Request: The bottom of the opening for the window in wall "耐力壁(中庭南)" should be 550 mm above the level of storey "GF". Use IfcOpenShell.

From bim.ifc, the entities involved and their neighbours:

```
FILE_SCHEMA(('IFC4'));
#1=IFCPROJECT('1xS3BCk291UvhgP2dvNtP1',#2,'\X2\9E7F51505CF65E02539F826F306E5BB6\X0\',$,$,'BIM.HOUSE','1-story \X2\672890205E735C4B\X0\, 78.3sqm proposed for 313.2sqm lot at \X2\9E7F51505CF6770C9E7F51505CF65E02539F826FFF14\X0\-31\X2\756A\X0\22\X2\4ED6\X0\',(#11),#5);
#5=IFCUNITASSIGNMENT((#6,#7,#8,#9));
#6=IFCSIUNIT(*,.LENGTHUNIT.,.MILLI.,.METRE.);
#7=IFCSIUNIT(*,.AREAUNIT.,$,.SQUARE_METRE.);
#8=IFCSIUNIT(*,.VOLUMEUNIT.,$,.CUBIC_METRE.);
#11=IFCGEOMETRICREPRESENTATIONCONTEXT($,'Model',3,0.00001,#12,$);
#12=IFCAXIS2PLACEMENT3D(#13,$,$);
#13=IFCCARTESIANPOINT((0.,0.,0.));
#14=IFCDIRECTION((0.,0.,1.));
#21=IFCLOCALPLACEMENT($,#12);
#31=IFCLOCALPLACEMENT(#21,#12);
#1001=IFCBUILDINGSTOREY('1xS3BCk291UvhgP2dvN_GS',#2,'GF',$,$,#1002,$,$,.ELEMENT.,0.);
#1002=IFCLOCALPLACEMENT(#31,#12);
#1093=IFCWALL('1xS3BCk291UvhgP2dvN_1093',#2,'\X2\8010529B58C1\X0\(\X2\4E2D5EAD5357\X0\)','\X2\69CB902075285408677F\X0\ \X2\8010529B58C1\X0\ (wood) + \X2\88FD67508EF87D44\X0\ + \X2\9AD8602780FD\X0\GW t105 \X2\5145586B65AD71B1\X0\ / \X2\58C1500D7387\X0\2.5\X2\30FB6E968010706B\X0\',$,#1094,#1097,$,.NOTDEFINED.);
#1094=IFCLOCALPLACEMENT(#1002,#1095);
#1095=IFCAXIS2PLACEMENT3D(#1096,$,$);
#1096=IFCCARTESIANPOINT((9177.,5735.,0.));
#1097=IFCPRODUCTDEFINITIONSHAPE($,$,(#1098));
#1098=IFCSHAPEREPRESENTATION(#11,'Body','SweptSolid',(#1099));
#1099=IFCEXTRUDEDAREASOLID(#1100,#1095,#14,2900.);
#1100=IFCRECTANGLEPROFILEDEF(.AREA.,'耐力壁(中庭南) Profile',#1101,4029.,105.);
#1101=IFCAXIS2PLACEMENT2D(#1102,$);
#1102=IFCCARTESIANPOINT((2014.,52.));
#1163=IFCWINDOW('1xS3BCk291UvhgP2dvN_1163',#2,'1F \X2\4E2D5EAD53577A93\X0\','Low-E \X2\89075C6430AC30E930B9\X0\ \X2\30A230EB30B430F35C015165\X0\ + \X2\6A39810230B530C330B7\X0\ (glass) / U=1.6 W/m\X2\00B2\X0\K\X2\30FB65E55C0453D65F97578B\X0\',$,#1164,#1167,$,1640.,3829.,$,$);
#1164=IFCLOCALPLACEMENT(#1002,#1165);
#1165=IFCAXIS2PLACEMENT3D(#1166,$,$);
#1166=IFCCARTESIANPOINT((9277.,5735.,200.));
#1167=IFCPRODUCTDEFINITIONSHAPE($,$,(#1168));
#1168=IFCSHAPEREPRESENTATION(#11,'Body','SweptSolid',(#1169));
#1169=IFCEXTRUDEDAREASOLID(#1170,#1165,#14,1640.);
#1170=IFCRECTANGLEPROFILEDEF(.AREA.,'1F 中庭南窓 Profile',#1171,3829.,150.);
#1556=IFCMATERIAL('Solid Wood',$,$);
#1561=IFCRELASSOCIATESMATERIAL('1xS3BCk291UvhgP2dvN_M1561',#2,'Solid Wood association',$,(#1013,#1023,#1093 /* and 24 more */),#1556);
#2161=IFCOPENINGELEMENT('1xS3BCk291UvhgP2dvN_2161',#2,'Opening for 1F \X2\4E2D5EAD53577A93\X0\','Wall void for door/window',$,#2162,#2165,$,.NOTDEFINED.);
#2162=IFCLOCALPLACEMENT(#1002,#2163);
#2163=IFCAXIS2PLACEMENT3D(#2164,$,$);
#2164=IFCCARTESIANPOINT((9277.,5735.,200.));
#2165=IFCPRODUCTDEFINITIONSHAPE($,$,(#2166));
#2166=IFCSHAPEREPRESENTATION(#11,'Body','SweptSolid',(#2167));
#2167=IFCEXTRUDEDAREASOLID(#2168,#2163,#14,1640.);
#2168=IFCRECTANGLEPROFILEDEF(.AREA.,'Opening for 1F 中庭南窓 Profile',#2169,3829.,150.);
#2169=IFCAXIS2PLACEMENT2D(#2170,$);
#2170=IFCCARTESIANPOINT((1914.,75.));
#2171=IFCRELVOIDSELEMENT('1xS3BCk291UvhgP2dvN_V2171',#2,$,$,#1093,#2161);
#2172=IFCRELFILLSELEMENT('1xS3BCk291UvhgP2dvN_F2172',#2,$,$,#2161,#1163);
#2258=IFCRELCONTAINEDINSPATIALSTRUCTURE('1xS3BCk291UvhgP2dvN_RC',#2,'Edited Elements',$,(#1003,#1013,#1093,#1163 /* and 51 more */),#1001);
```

```python
import numpy as np
import ifcopenshell
import ifcopenshell.api.geometry
import ifcopenshell.geom
import ifcopenshell.util.element
import ifcopenshell.util.placement
import ifcopenshell.util.shape
import ifcopenshell.util.unit

model = ifcopenshell.open("bim.ifc")
unit_scale = ifcopenshell.util.unit.calculate_unit_scale(model)

window = model.by_id(1163)
opening = window.FillsVoids[0].RelatingOpeningElement
storey = ifcopenshell.util.element.get_container(window, ifc_class="IfcBuildingStorey")
level = ifcopenshell.util.placement.get_local_placement(storey.ObjectPlacement)[2, 3]

# The opening's origin need not be at the sill, so measure its lowest point.
shape = ifcopenshell.geom.create_shape(ifcopenshell.geom.settings(), opening)
bottom = ifcopenshell.util.shape.get_shape_bottom_elevation(shape, shape.geometry) / unit_scale
dz = level + 0.55 / unit_scale - bottom

shift = np.array([0.0, 0.0, dz])
# The window is not placed relative to its opening, so move both.
for product in (opening, window):
    matrix = ifcopenshell.util.placement.get_local_placement(product.ObjectPlacement)
    matrix[:3, 3] += shift
    ifcopenshell.api.geometry.edit_object_placement(model, product=product, matrix=matrix, is_si=False)

print(f"moved by {dz * unit_scale:+.3f} m")

model.write("bim_rev.ifc")
```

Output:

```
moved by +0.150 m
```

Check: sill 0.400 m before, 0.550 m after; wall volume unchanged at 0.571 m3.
